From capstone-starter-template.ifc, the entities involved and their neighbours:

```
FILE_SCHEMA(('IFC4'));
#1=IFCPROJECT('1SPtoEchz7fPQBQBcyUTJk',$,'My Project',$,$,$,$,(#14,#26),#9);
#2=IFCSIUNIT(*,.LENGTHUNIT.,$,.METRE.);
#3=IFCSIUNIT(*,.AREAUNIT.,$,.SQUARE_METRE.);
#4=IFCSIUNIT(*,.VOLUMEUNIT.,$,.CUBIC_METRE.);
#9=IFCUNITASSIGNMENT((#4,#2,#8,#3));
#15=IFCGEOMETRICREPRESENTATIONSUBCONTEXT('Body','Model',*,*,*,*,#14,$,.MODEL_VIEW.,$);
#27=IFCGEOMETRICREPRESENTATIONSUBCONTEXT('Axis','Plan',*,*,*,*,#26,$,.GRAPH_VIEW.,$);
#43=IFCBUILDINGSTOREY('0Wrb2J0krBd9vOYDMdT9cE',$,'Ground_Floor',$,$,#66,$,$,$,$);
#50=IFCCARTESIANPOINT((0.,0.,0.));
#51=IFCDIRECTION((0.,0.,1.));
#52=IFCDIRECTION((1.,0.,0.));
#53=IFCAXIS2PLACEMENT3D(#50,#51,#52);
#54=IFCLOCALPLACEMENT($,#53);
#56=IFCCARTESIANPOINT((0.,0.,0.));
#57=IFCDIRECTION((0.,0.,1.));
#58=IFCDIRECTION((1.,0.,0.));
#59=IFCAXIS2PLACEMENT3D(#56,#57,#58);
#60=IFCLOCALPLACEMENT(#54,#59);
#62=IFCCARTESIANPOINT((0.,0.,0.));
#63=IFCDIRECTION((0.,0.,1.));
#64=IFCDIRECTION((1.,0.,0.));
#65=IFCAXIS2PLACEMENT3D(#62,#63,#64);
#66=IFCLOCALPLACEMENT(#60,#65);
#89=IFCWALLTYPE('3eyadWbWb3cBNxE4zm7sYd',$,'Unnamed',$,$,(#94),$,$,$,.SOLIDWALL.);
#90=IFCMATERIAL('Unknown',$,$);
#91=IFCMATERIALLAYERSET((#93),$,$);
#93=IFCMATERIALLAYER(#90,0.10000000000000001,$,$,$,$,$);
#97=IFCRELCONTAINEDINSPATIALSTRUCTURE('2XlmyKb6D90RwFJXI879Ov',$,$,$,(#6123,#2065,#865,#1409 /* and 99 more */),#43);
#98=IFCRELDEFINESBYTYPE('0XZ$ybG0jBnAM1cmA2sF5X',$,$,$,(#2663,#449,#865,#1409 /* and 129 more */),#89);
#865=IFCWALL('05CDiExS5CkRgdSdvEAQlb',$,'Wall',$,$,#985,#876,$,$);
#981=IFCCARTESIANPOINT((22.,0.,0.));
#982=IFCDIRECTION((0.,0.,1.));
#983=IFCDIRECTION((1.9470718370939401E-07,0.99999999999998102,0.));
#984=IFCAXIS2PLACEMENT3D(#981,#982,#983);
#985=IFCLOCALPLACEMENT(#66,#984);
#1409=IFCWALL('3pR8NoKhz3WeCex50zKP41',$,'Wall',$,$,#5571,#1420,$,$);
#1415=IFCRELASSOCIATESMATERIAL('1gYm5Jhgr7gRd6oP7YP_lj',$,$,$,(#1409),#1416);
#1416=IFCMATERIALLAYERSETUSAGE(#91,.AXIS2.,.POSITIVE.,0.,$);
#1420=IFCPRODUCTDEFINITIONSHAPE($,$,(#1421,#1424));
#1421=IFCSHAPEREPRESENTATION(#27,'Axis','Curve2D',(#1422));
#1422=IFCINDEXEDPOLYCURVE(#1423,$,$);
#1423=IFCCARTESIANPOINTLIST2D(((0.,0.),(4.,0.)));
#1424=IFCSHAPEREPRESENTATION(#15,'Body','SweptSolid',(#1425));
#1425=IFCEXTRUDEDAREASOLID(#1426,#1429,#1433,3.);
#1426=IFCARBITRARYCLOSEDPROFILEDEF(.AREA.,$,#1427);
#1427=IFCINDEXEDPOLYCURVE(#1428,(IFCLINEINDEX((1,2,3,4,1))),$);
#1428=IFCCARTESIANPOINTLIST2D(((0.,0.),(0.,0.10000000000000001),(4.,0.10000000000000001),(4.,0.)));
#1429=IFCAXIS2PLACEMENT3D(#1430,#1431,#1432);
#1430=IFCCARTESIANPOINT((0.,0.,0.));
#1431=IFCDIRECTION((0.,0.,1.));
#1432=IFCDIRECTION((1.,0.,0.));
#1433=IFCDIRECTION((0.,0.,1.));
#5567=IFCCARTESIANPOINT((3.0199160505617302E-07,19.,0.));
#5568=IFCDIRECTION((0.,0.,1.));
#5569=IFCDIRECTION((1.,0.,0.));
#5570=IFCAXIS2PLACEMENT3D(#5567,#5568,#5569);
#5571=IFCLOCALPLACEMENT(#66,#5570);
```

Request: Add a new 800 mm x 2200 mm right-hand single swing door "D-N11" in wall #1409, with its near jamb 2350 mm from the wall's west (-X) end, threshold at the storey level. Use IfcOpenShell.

```python
import numpy as np
import ifcopenshell
import ifcopenshell.api.feature
import ifcopenshell.api.geometry
import ifcopenshell.api.root
import ifcopenshell.api.spatial
import ifcopenshell.geom
import ifcopenshell.util.element
import ifcopenshell.util.placement
import ifcopenshell.util.representation
import ifcopenshell.util.shape
import ifcopenshell.util.unit

model = ifcopenshell.open("capstone-starter-template.ifc")
unit_scale = ifcopenshell.util.unit.calculate_unit_scale(model)
settings = ifcopenshell.geom.settings()


def volume(element):
    """Net volume in cubic metres, openings subtracted."""
    shape = ifcopenshell.geom.create_shape(settings, element)
    return ifcopenshell.util.shape.get_volume(shape.geometry)


wall = model.by_guid("3pR8NoKhz3WeCex50zKP41")
storey = ifcopenshell.util.element.get_container(wall, ifc_class="IfcBuildingStorey")
context = ifcopenshell.util.representation.get_context(model, "Model", "Body", "MODEL_VIEW")
before = volume(wall)

width, height, from_end, sill = 0.8, 2.2, 2.35, 0.0  # metres

# The wall runs along its own X axis, and the end named is its -X end.
wall_shape = ifcopenshell.geom.create_shape(settings, wall)
x, y, z = ifcopenshell.util.shape.get_vertices(wall_shape.geometry).T
start = x.min() + from_end
face, thickness = float(y.min()), float(y.max() - y.min())
wall_matrix = ifcopenshell.util.placement.get_local_placement(wall.ObjectPlacement)
level = ifcopenshell.util.placement.get_local_placement(storey.ObjectPlacement)[2, 3]


def in_wall(x, y):
    """Placement at x, y metres in the wall's axes, at sill height."""
    matrix = wall_matrix.copy()
    matrix[:, 3] = wall_matrix @ np.array([x / unit_scale, y / unit_scale, 0.0, 1.0])
    matrix[2, 3] = level + sill / unit_scale
    return matrix


# Opening: a box that overshoots both wall faces by 50 mm.
opening = ifcopenshell.api.root.create_entity(model, ifc_class="IfcOpeningElement", predefined_type="OPENING")
box = ifcopenshell.api.geometry.add_wall_representation(
    model, context=context, length=width, height=height, thickness=thickness + 0.1
)
ifcopenshell.api.geometry.assign_representation(model, product=opening, representation=box)
ifcopenshell.api.geometry.edit_object_placement(model, product=opening, matrix=in_wall(start, face - 0.05), is_si=False)
ifcopenshell.api.feature.add_feature(model, feature=opening, element=wall)

door = ifcopenshell.api.root.create_entity(model, ifc_class="IfcDoor", name="D-N11", predefined_type="DOOR")
door.OverallWidth, door.OverallHeight = width / unit_scale, height / unit_scale
door.OperationType = "SINGLE_SWING_RIGHT"
body = ifcopenshell.api.geometry.add_door_representation(
    model,
    context=context,
    overall_width=door.OverallWidth,
    overall_height=door.OverallHeight,
    operation_type="SINGLE_SWING_RIGHT",
    lining_properties={"LiningDepth": thickness / unit_scale, "ThresholdDepth": thickness / unit_scale},
)
ifcopenshell.api.geometry.assign_representation(model, product=door, representation=body)
ifcopenshell.api.spatial.assign_container(model, products=[door], relating_structure=storey)
ifcopenshell.api.feature.add_filling(model, opening=opening, element=door)

# The lining spans the wall, so the door starts at the wall face.
ifcopenshell.api.geometry.edit_object_placement(model, product=door, matrix=in_wall(start, face), is_si=False)

after = volume(wall)

print(f"wall volume {before:.3f} -> {after:.3f} m3")

model.write("capstone-starter-template-out.ifc")
```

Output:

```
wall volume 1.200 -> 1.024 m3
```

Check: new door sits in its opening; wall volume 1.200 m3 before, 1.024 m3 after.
